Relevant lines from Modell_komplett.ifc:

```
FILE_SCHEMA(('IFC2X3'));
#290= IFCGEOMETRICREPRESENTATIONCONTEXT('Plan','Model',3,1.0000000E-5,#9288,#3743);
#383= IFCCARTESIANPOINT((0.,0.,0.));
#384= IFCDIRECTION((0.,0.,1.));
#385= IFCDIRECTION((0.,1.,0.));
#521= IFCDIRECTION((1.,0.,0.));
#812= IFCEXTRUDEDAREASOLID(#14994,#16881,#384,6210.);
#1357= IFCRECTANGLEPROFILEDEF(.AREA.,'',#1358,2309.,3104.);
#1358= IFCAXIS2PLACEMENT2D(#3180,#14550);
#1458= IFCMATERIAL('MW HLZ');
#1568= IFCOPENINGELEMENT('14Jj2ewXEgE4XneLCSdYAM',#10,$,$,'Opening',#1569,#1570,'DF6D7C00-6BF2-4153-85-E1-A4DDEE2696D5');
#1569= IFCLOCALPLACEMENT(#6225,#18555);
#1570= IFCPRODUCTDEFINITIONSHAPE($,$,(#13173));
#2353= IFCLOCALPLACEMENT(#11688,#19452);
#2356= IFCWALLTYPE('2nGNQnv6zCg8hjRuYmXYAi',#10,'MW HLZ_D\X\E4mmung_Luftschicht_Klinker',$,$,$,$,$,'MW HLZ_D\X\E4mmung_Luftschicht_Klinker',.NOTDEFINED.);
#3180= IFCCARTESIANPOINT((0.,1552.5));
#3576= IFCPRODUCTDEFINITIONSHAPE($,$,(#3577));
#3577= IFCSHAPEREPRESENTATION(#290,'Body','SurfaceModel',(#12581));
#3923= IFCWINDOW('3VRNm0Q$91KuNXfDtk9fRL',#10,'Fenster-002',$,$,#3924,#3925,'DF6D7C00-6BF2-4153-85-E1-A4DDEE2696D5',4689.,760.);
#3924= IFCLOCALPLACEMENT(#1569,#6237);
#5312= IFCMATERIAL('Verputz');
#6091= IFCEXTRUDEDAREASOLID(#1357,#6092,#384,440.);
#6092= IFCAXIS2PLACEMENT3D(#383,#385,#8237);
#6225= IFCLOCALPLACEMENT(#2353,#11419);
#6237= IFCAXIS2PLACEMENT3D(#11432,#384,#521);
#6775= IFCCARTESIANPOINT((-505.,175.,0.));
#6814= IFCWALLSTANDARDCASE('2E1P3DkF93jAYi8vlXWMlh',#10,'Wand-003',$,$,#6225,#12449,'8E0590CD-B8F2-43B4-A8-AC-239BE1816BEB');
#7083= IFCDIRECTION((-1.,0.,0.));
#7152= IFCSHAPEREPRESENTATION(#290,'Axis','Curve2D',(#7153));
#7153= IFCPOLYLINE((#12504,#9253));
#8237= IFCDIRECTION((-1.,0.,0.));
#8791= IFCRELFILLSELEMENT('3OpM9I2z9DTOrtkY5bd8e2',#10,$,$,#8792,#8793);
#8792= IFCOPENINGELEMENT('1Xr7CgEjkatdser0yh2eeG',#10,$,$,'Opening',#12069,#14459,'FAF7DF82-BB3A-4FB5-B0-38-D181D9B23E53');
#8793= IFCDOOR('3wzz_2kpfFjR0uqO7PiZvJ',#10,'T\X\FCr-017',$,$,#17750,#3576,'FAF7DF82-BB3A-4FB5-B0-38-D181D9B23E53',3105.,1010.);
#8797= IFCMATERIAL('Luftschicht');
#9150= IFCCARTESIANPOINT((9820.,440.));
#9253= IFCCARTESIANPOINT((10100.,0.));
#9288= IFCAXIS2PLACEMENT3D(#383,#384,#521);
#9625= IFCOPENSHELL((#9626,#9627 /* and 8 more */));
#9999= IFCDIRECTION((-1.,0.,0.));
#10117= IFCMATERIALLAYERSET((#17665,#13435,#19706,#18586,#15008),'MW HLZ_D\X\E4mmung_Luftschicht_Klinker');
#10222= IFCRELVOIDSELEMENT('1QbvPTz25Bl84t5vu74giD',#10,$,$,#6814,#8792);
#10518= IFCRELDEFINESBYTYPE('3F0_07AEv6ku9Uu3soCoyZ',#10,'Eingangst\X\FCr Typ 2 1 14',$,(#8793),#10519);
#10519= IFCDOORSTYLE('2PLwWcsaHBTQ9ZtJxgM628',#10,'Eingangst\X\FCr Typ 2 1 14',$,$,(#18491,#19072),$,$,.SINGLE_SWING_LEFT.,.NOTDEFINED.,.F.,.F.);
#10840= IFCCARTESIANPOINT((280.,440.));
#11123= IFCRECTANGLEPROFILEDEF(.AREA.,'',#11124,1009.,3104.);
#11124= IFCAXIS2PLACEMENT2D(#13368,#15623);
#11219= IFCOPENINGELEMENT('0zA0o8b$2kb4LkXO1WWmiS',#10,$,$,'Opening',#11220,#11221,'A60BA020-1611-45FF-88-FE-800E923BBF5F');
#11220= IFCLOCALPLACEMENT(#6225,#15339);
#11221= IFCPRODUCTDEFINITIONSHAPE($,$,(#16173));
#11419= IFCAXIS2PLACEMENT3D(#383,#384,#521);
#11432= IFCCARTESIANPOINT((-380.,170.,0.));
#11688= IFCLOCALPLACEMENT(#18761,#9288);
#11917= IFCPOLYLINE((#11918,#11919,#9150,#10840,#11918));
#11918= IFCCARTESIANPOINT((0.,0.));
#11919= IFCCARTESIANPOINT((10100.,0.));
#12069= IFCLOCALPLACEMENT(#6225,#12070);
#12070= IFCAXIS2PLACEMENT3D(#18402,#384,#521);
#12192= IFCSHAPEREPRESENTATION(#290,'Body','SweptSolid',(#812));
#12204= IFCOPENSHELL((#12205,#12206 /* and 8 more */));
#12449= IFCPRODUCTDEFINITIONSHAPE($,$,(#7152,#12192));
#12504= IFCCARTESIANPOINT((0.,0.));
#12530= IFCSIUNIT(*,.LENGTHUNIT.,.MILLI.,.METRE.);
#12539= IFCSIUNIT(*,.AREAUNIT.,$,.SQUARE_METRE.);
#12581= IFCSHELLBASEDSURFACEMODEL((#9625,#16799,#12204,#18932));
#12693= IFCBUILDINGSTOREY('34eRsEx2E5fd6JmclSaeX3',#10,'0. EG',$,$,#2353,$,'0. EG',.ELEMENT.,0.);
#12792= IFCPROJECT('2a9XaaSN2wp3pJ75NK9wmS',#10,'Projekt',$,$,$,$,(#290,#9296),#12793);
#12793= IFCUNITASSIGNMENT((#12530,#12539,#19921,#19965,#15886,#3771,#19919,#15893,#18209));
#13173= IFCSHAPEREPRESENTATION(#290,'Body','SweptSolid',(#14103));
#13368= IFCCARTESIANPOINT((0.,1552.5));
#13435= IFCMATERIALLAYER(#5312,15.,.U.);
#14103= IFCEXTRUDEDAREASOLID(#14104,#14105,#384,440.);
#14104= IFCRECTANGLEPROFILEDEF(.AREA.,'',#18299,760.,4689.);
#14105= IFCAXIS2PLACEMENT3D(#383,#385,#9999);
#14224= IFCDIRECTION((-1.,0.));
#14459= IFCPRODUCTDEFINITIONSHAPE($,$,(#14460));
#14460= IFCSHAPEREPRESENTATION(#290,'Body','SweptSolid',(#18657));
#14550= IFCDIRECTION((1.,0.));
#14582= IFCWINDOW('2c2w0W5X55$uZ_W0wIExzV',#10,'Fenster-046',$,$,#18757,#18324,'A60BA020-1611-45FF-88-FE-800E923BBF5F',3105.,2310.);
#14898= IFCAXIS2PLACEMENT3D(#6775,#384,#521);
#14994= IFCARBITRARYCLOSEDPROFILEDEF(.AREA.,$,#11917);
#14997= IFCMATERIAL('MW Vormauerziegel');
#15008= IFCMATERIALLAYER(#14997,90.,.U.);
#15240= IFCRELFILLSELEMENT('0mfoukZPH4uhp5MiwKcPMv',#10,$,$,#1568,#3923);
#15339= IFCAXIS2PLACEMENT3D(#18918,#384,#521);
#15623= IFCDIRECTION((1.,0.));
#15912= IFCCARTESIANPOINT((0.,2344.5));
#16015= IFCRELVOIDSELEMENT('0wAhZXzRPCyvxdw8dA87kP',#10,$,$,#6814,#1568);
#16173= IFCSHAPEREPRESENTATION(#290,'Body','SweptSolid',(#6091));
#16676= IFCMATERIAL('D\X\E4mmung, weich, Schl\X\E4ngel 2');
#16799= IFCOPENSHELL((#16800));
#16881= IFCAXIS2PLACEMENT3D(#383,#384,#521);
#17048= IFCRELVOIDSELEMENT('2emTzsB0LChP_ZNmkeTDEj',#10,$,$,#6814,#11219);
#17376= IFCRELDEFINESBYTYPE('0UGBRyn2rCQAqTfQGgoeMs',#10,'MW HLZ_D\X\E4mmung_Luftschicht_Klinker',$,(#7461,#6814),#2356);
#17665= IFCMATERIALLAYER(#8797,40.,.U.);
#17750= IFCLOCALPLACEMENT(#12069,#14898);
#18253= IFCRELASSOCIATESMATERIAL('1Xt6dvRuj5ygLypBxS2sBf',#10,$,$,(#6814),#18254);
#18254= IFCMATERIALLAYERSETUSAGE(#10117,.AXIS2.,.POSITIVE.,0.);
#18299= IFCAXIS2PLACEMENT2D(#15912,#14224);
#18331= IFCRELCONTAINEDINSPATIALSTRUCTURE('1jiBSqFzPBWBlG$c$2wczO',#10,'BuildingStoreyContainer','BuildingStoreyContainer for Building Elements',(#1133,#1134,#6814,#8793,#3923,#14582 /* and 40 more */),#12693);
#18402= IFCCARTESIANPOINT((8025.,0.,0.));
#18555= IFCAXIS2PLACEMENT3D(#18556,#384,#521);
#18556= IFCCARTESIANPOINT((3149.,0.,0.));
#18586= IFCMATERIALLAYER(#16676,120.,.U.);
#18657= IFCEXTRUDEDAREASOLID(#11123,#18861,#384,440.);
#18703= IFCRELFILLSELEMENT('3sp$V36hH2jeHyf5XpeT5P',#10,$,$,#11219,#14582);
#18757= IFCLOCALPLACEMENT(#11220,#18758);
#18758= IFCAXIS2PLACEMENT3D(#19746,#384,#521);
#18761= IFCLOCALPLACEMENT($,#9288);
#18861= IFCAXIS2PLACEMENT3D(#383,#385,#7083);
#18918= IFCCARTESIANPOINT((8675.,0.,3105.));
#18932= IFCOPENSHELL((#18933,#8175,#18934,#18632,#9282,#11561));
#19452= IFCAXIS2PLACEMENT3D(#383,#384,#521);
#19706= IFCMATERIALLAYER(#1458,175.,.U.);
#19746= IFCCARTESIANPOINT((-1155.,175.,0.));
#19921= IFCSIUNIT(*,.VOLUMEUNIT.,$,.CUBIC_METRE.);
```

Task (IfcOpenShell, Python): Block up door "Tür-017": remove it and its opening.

```python
import ifcopenshell
import ifcopenshell.api.feature
import ifcopenshell.api.root
import ifcopenshell.geom
import ifcopenshell.util.shape

model = ifcopenshell.open("Modell_komplett.ifc")
settings = ifcopenshell.geom.settings()


def volume(element):
    """Net volume in cubic metres, openings subtracted."""
    shape = ifcopenshell.geom.create_shape(settings, element)
    return ifcopenshell.util.shape.get_volume(shape.geometry)


door = model.by_id(8793)
opening = door.FillsVoids[0].RelatingOpeningElement
wall = opening.VoidsElements[0].RelatingBuildingElement
before = volume(wall)

ifcopenshell.api.root.remove_product(model, product=door)
ifcopenshell.api.feature.remove_feature(model, feature=opening)

after = volume(wall)

print(f"wall volume {before:.3f} -> {after:.3f} m3")

model.write("Modell_komplett_updated.ifc")
```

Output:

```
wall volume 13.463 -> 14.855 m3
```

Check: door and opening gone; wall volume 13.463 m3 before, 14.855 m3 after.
